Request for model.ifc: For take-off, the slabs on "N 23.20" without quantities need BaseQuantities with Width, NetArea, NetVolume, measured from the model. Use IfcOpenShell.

First a look at what the model holds.

```python
import ifcopenshell
import ifcopenshell.util.element
import ifcopenshell.util.unit

model = ifcopenshell.open("model.ifc")
print(model.schema)
for unit_type in ("LENGTHUNIT", "AREAUNIT", "VOLUMEUNIT"):
    print(unit_type, ifcopenshell.util.unit.calculate_unit_scale(model, unit_type))
storey = next(s for s in model.by_type("IfcBuildingStorey") if s.Name == "N 23.20")
slabs = [e for e in ifcopenshell.util.element.get_decomposition(storey) if e.is_a("IfcSlab")]
for e in sorted(slabs, key=lambda e: e.id()):
    print(e.id(), e.is_a(), e.Name, list(ifcopenshell.util.element.get_psets(e, qtos_only=True)), sep=" | ")
```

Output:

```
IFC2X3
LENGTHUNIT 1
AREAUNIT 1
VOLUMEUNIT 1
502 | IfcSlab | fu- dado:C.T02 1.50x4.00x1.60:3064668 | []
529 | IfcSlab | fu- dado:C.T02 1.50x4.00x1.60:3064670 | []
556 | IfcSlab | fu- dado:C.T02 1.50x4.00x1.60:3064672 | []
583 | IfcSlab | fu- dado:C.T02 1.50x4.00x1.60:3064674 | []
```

```python
import ifcopenshell
import ifcopenshell.api.pset
import ifcopenshell.geom
import ifcopenshell.util.element
import ifcopenshell.util.shape
import ifcopenshell.util.unit

model = ifcopenshell.open("model.ifc")
unit_scale = ifcopenshell.util.unit.calculate_unit_scale(model)
area_scale = ifcopenshell.util.unit.calculate_unit_scale(model, "AREAUNIT")
volume_scale = ifcopenshell.util.unit.calculate_unit_scale(model, "VOLUMEUNIT")
settings = ifcopenshell.geom.settings()

storey = next(s for s in model.by_type("IfcBuildingStorey") if s.Name == "N 23.20")
slabs = [e for e in ifcopenshell.util.element.get_decomposition(storey) if e.is_a("IfcSlab")]

for e in sorted(slabs, key=lambda e: e.id()):
    if ifcopenshell.util.element.get_psets(e, qtos_only=True, should_inherit=False):
        continue
    # Geometry comes back in metres, in the element's own axes.
    shape = ifcopenshell.geom.create_shape(settings, e)
    values = {
        "Width": ifcopenshell.util.shape.get_z(shape.geometry) / unit_scale,
        "NetArea": ifcopenshell.util.shape.get_footprint_area(shape.geometry) / area_scale,
        "NetVolume": ifcopenshell.util.shape.get_volume(shape.geometry) / volume_scale,
    }
    qto = ifcopenshell.api.pset.add_qto(model, product=e, name="BaseQuantities")
    ifcopenshell.api.pset.edit_qto(model, qto=qto, properties=values)
    print(e.id(), {k: round(v, 3) for k, v in values.items()})

model.write("model_updated.ifc")
```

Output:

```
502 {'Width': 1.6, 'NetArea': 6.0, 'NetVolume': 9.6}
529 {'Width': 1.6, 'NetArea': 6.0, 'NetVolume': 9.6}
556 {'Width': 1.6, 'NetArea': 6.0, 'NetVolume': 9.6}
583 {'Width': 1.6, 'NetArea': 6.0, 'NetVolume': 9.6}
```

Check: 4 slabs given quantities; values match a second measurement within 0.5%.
